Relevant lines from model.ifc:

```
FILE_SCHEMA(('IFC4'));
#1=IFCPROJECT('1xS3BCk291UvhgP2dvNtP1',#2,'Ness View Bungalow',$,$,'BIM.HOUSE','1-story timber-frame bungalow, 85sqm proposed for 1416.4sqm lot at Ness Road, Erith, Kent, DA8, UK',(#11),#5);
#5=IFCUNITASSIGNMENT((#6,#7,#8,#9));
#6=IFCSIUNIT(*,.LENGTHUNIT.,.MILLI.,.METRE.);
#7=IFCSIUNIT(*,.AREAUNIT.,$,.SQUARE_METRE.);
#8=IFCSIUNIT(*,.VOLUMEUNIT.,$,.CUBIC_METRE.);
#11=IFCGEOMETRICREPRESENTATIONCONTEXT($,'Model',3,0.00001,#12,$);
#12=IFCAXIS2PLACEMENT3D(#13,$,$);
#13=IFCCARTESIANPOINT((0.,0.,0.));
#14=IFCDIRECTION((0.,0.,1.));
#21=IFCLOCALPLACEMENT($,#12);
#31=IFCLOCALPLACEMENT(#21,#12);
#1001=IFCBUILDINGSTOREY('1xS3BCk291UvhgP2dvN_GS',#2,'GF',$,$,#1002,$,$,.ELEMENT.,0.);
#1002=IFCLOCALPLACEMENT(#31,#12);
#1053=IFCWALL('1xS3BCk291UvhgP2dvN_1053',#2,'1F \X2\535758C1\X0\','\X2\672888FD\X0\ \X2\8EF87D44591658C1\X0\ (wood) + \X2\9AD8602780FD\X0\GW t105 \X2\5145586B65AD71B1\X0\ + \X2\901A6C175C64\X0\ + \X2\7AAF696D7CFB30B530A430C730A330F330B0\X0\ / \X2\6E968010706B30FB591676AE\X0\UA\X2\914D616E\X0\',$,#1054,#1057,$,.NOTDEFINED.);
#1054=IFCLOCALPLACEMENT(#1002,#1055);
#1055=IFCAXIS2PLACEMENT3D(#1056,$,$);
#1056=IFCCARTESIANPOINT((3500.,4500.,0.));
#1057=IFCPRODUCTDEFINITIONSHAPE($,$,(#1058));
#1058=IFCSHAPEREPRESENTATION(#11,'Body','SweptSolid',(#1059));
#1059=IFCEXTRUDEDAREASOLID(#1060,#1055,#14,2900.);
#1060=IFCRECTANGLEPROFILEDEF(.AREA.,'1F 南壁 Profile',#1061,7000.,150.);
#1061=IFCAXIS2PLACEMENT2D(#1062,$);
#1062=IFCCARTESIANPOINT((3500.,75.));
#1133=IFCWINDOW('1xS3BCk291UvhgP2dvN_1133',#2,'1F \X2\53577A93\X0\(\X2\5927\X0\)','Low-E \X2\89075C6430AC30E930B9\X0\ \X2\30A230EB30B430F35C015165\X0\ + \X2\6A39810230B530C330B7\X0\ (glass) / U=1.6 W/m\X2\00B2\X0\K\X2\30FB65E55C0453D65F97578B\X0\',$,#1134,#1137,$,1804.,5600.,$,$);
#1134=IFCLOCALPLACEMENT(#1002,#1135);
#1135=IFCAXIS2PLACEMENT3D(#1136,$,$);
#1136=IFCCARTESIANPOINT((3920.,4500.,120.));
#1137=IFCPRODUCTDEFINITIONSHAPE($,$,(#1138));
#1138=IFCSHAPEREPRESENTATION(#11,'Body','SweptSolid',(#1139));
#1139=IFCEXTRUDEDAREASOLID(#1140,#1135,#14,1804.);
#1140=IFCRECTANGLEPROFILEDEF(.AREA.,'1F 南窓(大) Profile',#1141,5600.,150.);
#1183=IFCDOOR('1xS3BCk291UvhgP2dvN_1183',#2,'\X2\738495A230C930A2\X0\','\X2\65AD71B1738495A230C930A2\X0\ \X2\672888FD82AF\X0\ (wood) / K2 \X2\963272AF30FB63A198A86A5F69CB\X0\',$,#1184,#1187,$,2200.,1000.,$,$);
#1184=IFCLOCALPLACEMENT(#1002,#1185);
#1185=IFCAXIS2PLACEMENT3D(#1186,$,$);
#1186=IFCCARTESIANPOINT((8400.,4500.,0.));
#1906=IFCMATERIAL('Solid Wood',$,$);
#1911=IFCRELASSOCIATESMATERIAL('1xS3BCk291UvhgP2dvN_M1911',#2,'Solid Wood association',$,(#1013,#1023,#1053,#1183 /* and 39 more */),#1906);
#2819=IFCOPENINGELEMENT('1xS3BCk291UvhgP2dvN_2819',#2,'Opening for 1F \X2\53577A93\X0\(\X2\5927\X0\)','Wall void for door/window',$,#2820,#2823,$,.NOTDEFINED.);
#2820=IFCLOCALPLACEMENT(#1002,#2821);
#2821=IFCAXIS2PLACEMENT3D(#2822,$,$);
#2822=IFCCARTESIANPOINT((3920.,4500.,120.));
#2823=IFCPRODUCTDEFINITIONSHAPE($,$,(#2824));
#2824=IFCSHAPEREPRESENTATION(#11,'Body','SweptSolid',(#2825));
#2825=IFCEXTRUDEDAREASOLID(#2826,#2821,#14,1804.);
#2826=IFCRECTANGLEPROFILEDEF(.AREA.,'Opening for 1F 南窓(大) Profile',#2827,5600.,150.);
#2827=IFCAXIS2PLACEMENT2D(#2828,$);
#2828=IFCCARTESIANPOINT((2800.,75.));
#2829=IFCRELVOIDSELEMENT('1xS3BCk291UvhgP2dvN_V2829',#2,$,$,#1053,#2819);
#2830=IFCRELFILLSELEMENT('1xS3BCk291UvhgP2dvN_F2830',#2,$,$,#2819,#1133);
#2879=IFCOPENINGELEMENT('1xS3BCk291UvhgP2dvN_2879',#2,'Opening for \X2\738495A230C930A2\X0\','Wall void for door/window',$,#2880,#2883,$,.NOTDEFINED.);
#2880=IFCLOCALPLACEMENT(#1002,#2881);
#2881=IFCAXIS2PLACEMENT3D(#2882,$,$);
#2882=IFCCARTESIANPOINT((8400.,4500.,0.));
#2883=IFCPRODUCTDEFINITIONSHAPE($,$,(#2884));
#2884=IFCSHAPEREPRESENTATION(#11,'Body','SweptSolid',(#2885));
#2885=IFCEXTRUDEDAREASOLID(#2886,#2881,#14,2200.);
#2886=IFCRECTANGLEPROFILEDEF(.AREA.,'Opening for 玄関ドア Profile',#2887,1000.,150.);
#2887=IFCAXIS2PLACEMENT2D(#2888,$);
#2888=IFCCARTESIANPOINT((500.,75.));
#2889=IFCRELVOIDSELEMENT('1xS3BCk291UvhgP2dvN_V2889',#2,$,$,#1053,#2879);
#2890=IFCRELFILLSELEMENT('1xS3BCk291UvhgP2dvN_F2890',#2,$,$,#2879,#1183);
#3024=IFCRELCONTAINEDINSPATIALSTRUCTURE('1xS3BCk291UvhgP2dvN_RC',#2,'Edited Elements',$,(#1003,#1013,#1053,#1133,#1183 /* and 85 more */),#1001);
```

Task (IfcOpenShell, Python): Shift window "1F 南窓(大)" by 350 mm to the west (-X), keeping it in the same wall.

```python
import ifcopenshell
import ifcopenshell.api.geometry
import ifcopenshell.util.placement
import ifcopenshell.util.unit

model = ifcopenshell.open("model.ifc")
unit_scale = ifcopenshell.util.unit.calculate_unit_scale(model)

window = model.by_guid("1xS3BCk291UvhgP2dvN_1133")
opening = window.FillsVoids[0].RelatingOpeningElement
wall = opening.VoidsElements[0].RelatingBuildingElement

wall_matrix = ifcopenshell.util.placement.get_local_placement(wall.ObjectPlacement)
shift = wall_matrix[:3, 0] * -0.35 / unit_scale
before = ifcopenshell.util.placement.get_local_placement(window.ObjectPlacement)[:3, 3].copy()

# The window is not placed relative to its opening, so move both.
for product in (opening, window):
    matrix = ifcopenshell.util.placement.get_local_placement(product.ObjectPlacement)
    matrix[:3, 3] += shift
    ifcopenshell.api.geometry.edit_object_placement(model, product=product, matrix=matrix, is_si=False)

after = ifcopenshell.util.placement.get_local_placement(window.ObjectPlacement)[:3, 3]
print("window moved by", (after - before).round(3) + 0.0)

model.write("model_v2.ifc")
```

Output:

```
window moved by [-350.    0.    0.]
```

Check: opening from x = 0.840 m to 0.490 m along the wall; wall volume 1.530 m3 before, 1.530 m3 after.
